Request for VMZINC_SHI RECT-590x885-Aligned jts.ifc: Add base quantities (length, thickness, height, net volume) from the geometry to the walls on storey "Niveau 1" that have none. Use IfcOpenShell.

First a look at what the model holds.

```python
import ifcopenshell
import ifcopenshell.util.element
import ifcopenshell.util.unit

model = ifcopenshell.open("VMZINC_SHI RECT-590x885-Aligned jts.ifc")
print(model.schema)
for unit_type in ("LENGTHUNIT", "AREAUNIT", "VOLUMEUNIT"):
    print(unit_type, ifcopenshell.util.unit.calculate_unit_scale(model, unit_type))
storey = next(s for s in model.by_type("IfcBuildingStorey") if s.Name == "Niveau 1")
walls = [e for e in ifcopenshell.util.element.get_decomposition(storey) if e.is_a("IfcWall")]
for e in sorted(walls, key=lambda e: e.id()):
    print(e.id(), e.is_a(), e.Name, list(ifcopenshell.util.element.get_psets(e, qtos_only=True)), sep=" | ")
```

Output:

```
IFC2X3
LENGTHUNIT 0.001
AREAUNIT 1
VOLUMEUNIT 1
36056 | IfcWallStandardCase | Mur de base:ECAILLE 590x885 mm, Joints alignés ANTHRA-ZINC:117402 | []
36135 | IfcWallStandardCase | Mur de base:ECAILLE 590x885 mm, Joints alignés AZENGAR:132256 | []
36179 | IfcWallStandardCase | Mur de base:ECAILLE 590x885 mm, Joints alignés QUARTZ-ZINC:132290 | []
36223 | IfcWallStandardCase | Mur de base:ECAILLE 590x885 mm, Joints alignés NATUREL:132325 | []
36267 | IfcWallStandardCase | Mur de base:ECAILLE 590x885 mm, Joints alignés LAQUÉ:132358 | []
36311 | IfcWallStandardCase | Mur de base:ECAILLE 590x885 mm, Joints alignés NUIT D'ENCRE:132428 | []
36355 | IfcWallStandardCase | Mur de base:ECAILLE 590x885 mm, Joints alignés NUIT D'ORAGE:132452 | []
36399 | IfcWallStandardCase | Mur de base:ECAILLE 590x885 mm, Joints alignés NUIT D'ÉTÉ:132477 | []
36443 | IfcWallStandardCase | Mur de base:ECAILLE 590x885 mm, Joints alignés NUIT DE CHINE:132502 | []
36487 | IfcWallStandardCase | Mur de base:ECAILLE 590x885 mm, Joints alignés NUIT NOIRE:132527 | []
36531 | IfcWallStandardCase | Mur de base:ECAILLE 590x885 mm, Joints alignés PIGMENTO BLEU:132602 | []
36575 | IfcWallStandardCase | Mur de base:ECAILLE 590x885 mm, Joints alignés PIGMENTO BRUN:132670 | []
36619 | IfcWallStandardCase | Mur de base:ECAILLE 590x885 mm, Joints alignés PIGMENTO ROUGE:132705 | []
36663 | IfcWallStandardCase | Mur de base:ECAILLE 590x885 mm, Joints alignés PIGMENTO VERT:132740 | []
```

```python
import ifcopenshell
import ifcopenshell.api.pset
import ifcopenshell.geom
import ifcopenshell.util.element
import ifcopenshell.util.shape
import ifcopenshell.util.unit

model = ifcopenshell.open("VMZINC_SHI RECT-590x885-Aligned jts.ifc")
unit_scale = ifcopenshell.util.unit.calculate_unit_scale(model)
volume_scale = ifcopenshell.util.unit.calculate_unit_scale(model, "VOLUMEUNIT")
settings = ifcopenshell.geom.settings()

storey = next(s for s in model.by_type("IfcBuildingStorey") if s.Name == "Niveau 1")
walls = [e for e in ifcopenshell.util.element.get_decomposition(storey) if e.is_a("IfcWall")]

for e in sorted(walls, key=lambda e: e.id()):
    if ifcopenshell.util.element.get_psets(e, qtos_only=True, should_inherit=False):
        continue
    # Geometry comes back in metres, in the element's own axes.
    shape = ifcopenshell.geom.create_shape(settings, e)
    values = {
        "Length": ifcopenshell.util.shape.get_x(shape.geometry) / unit_scale,
        "Width": ifcopenshell.util.shape.get_y(shape.geometry) / unit_scale,
        "Height": ifcopenshell.util.shape.get_z(shape.geometry) / unit_scale,
        "NetVolume": ifcopenshell.util.shape.get_volume(shape.geometry) / volume_scale,
    }
    qto = ifcopenshell.api.pset.add_qto(model, product=e, name="BaseQuantities")
    ifcopenshell.api.pset.edit_qto(model, qto=qto, properties=values)
    print(e.id(), {k: round(v, 3) for k, v in values.items()})

model.write("VMZINC_SHI RECT-590x885-Aligned jts_v2.ifc")
```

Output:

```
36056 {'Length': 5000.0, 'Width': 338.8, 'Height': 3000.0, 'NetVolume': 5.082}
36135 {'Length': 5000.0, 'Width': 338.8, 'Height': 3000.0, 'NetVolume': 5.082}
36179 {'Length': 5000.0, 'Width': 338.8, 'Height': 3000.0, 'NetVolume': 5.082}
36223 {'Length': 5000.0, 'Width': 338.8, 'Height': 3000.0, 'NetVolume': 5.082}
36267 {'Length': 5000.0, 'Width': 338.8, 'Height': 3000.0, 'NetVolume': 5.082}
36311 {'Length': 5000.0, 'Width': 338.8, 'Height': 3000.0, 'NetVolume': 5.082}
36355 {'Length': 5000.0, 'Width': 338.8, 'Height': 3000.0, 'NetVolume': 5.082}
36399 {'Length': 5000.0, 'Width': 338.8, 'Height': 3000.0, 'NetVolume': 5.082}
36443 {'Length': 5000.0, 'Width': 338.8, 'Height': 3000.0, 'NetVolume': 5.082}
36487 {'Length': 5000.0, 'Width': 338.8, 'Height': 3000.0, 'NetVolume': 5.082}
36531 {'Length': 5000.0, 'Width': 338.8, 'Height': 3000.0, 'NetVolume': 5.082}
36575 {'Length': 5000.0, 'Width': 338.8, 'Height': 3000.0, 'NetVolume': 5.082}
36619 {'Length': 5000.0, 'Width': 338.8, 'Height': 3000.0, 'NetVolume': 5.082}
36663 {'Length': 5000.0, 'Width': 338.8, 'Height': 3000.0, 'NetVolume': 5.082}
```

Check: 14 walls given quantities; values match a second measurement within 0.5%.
